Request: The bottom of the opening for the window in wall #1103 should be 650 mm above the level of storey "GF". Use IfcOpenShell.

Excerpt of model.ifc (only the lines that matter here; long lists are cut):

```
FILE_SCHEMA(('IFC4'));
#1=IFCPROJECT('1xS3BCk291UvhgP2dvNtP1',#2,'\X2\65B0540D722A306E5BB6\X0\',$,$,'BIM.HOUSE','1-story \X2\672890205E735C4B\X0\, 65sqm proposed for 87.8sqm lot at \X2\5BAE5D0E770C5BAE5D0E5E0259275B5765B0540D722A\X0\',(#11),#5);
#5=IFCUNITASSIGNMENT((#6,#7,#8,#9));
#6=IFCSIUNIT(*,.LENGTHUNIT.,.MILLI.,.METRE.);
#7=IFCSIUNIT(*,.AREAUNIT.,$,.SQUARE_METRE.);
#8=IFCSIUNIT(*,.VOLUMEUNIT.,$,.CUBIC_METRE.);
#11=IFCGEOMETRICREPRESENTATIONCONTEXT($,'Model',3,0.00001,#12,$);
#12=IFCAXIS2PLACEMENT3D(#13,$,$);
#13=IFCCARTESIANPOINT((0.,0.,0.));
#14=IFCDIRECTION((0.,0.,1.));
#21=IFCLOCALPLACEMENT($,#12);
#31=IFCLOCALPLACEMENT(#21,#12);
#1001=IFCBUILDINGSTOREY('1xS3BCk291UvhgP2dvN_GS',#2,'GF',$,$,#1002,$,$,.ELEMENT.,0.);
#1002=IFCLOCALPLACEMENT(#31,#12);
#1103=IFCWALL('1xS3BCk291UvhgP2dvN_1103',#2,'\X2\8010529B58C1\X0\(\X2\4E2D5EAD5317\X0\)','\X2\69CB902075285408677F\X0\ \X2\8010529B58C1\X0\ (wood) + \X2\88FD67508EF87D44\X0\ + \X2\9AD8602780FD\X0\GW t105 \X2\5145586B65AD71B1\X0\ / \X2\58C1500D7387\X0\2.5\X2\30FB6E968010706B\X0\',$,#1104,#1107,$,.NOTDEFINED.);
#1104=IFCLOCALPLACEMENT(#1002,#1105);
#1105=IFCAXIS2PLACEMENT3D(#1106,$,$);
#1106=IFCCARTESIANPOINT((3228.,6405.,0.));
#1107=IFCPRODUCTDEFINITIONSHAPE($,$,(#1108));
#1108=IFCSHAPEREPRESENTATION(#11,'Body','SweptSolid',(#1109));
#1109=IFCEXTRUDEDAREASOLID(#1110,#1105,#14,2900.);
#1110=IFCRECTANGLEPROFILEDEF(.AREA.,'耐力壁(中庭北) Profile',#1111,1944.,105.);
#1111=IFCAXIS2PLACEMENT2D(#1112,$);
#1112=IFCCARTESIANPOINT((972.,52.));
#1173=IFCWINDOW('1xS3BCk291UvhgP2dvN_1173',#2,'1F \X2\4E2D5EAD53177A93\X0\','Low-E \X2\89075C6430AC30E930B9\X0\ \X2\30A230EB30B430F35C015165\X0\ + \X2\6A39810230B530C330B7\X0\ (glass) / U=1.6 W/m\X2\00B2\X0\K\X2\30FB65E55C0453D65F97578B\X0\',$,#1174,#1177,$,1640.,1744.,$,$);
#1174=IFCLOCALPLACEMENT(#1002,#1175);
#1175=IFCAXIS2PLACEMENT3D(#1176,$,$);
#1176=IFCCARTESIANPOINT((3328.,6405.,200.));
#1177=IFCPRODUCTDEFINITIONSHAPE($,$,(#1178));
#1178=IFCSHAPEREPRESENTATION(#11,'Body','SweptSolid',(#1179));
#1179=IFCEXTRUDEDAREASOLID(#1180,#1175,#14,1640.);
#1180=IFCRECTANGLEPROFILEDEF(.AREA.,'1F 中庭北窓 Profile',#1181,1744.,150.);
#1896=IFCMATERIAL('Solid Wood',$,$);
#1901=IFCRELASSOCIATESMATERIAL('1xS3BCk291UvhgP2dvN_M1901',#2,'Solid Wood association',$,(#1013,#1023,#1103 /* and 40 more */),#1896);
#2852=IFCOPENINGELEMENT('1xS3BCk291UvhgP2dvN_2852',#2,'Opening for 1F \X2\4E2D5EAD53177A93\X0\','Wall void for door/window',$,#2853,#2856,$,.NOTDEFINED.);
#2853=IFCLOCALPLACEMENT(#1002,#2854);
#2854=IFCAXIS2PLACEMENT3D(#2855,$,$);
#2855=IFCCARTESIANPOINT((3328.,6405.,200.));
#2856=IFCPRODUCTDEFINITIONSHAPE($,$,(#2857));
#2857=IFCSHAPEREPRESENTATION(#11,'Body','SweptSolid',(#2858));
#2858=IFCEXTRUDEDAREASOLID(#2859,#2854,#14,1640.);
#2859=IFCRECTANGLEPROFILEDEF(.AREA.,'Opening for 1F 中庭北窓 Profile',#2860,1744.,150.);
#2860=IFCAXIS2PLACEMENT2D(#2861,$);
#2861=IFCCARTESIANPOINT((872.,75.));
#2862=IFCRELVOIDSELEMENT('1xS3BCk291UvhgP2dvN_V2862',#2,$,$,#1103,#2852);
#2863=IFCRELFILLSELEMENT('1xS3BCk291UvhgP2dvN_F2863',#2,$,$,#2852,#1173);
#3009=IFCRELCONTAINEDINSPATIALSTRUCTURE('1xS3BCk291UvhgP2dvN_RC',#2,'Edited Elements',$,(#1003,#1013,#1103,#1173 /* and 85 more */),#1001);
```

```python
import numpy as np
import ifcopenshell
import ifcopenshell.api.geometry
import ifcopenshell.geom
import ifcopenshell.util.element
import ifcopenshell.util.placement
import ifcopenshell.util.shape
import ifcopenshell.util.unit

model = ifcopenshell.open("model.ifc")
unit_scale = ifcopenshell.util.unit.calculate_unit_scale(model)

window = model.by_id(1173)
opening = window.FillsVoids[0].RelatingOpeningElement
storey = ifcopenshell.util.element.get_container(window, ifc_class="IfcBuildingStorey")
level = ifcopenshell.util.placement.get_local_placement(storey.ObjectPlacement)[2, 3]

# The opening's origin need not be at the sill, so measure its lowest point.
shape = ifcopenshell.geom.create_shape(ifcopenshell.geom.settings(), opening)
bottom = ifcopenshell.util.shape.get_shape_bottom_elevation(shape, shape.geometry) / unit_scale
dz = level + 650.0 - bottom

shift = np.array([0.0, 0.0, dz])
# The window is not placed relative to its opening, so move both.
for product in (opening, window):
    matrix = ifcopenshell.util.placement.get_local_placement(product.ObjectPlacement)
    matrix[:3, 3] += shift
    ifcopenshell.api.geometry.edit_object_placement(model, product=product, matrix=matrix, is_si=False)

print(f"moved by {dz * unit_scale:+.3f} m")

model.write("model_edited.ifc")
```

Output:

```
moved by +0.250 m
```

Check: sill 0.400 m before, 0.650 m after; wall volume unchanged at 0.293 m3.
